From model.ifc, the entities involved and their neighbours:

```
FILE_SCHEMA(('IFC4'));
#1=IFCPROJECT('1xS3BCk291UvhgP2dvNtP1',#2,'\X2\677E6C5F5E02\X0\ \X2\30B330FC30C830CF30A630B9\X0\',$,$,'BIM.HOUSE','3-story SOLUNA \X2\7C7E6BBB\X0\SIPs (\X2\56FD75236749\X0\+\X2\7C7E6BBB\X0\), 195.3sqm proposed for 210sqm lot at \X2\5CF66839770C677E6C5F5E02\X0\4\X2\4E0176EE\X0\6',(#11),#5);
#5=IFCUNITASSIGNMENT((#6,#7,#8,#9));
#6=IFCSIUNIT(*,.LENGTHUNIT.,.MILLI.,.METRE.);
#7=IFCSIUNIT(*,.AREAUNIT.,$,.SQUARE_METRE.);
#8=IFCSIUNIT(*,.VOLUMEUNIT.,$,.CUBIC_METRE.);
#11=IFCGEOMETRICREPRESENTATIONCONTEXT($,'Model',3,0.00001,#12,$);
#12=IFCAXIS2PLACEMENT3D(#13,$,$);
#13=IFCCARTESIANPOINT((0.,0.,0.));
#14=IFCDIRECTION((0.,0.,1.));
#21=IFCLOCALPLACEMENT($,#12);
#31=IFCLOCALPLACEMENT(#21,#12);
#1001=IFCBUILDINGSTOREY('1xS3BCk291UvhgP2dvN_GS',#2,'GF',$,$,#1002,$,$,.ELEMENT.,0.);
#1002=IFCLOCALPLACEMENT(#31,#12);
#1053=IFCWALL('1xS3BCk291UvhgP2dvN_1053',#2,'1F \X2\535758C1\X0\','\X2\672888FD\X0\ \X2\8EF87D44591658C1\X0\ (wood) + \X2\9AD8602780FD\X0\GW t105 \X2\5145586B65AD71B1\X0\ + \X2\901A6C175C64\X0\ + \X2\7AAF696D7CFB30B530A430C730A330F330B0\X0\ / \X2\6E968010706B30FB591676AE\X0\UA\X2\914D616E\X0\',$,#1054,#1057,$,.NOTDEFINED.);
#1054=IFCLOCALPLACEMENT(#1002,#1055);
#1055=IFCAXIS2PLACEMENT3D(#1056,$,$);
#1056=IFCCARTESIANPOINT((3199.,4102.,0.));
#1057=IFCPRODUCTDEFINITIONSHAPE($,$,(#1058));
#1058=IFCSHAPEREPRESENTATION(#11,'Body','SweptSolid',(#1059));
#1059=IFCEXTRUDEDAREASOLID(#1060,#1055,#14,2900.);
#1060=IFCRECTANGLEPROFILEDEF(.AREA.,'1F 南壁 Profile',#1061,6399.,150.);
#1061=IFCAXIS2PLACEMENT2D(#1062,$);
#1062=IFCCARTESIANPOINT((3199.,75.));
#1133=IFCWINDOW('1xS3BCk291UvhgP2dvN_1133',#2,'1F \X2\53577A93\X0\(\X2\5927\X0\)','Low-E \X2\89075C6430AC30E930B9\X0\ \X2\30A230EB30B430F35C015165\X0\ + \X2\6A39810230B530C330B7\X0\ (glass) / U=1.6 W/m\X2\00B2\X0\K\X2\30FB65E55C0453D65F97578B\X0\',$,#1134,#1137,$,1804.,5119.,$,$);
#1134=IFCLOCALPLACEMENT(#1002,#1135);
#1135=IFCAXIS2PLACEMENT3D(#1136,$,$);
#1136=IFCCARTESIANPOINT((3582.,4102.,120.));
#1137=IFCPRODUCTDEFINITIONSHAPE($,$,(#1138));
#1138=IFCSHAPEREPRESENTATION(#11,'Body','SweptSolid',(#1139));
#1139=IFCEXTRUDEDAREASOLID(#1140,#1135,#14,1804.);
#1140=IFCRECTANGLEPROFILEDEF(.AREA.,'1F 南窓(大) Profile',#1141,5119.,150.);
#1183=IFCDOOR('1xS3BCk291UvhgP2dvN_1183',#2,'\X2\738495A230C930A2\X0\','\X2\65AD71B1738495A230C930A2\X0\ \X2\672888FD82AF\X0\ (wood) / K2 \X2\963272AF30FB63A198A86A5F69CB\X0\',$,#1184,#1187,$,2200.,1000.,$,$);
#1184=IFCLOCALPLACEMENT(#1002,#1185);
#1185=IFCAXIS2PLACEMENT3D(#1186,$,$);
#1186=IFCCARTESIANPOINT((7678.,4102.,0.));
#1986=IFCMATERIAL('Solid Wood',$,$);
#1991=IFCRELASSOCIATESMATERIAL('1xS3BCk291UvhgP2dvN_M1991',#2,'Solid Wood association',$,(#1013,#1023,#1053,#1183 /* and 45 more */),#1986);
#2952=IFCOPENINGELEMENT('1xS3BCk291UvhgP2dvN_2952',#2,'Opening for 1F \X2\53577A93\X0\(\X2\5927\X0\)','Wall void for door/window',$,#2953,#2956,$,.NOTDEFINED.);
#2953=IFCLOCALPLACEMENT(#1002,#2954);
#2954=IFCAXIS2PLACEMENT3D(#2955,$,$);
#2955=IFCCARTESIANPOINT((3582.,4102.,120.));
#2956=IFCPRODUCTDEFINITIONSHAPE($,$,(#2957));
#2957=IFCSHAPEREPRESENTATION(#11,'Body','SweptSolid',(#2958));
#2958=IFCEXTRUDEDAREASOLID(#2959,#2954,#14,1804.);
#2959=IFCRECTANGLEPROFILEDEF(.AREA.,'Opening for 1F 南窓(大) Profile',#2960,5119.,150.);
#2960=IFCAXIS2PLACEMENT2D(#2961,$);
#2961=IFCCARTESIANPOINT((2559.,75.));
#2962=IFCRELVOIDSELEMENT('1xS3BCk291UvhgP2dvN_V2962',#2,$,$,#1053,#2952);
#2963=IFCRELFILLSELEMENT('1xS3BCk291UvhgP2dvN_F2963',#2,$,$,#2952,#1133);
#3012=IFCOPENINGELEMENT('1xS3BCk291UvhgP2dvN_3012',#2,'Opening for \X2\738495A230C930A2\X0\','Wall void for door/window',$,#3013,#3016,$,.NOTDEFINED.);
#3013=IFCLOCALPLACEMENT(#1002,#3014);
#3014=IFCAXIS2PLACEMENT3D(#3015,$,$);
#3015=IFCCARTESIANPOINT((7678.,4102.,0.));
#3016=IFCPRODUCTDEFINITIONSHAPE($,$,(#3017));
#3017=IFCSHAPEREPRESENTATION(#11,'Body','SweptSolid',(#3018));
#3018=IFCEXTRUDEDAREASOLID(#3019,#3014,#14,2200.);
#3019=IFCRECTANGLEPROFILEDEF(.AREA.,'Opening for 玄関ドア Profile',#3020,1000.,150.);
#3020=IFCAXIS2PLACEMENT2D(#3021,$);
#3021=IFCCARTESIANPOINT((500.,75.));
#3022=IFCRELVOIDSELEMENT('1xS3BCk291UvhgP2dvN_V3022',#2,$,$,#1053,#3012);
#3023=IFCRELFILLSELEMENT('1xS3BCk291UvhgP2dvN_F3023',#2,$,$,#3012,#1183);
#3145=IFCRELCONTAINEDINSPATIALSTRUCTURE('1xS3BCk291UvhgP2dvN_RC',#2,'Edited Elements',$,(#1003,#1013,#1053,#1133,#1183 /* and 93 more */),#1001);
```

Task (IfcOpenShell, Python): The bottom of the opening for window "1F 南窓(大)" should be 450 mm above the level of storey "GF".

```python
import numpy as np
import ifcopenshell
import ifcopenshell.api.geometry
import ifcopenshell.geom
import ifcopenshell.util.element
import ifcopenshell.util.placement
import ifcopenshell.util.shape
import ifcopenshell.util.unit

model = ifcopenshell.open("model.ifc")
unit_scale = ifcopenshell.util.unit.calculate_unit_scale(model)

window = model.by_guid("1xS3BCk291UvhgP2dvN_1133")
opening = window.FillsVoids[0].RelatingOpeningElement
storey = ifcopenshell.util.element.get_container(window, ifc_class="IfcBuildingStorey")
level = ifcopenshell.util.placement.get_local_placement(storey.ObjectPlacement)[2, 3]

# The opening's origin need not be at the sill, so measure its lowest point.
shape = ifcopenshell.geom.create_shape(ifcopenshell.geom.settings(), opening)
bottom = ifcopenshell.util.shape.get_shape_bottom_elevation(shape, shape.geometry) / unit_scale
dz = level + 450.0 - bottom

shift = np.array([0.0, 0.0, dz])
# The window is not placed relative to its opening, so move both.
for product in (opening, window):
    matrix = ifcopenshell.util.placement.get_local_placement(product.ObjectPlacement)
    matrix[:3, 3] += shift
    ifcopenshell.api.geometry.edit_object_placement(model, product=product, matrix=matrix, is_si=False)

print(f"moved by {dz * unit_scale:+.3f} m")

model.write("model_edited.ifc")
```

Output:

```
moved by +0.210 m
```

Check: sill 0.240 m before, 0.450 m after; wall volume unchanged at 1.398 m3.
